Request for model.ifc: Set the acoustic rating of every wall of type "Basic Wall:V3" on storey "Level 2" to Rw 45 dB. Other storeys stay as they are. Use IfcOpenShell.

First a look at what the model holds.

```python
import ifcopenshell
import ifcopenshell.util.element

model = ifcopenshell.open("model.ifc")
print(model.schema)
storey = next(s for s in model.by_type("IfcBuildingStorey") if s.Name == "Level 2")
walls = [e for e in ifcopenshell.util.element.get_decomposition(storey) if e.is_a("IfcWall")]
seen = {}
for e in walls:
    element_type = ifcopenshell.util.element.get_type(e)
    key = (element_type.Name if element_type != e and element_type else None, ifcopenshell.util.element.get_pset(e, "Pset_WallCommon", "AcousticRating"))
    seen[key] = seen.get(key, 0) + 1
for (name, value), count in sorted(seen.items(), key=str):
    print(count, "x", name, "|", value)
```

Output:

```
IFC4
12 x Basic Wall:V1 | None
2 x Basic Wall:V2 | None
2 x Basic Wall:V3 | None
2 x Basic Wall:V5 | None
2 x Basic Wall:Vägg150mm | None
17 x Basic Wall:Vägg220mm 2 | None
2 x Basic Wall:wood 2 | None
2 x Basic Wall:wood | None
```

```python
import ifcopenshell
import ifcopenshell.api.pset
import ifcopenshell.util.element

model = ifcopenshell.open("model.ifc")

storey = next(s for s in model.by_type("IfcBuildingStorey") if s.Name == "Level 2")
walls = [e for e in ifcopenshell.util.element.get_decomposition(storey) if e.is_a("IfcWall")]

count = 0
for e in walls:
    element_type = ifcopenshell.util.element.get_type(e)
    if element_type in (None, e) or element_type.Name != "Basic Wall:V3":
        continue
    # add_pset returns the element's existing set when there is one.
    pset = ifcopenshell.api.pset.add_pset(model, product=e, name="Pset_WallCommon")
    ifcopenshell.api.pset.edit_pset(model, pset=pset, properties={"AcousticRating": "Rw 45 dB"})
    count += 1

print(count, "walls updated")

model.write("model_updated.ifc")
```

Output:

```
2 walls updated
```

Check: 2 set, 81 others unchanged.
